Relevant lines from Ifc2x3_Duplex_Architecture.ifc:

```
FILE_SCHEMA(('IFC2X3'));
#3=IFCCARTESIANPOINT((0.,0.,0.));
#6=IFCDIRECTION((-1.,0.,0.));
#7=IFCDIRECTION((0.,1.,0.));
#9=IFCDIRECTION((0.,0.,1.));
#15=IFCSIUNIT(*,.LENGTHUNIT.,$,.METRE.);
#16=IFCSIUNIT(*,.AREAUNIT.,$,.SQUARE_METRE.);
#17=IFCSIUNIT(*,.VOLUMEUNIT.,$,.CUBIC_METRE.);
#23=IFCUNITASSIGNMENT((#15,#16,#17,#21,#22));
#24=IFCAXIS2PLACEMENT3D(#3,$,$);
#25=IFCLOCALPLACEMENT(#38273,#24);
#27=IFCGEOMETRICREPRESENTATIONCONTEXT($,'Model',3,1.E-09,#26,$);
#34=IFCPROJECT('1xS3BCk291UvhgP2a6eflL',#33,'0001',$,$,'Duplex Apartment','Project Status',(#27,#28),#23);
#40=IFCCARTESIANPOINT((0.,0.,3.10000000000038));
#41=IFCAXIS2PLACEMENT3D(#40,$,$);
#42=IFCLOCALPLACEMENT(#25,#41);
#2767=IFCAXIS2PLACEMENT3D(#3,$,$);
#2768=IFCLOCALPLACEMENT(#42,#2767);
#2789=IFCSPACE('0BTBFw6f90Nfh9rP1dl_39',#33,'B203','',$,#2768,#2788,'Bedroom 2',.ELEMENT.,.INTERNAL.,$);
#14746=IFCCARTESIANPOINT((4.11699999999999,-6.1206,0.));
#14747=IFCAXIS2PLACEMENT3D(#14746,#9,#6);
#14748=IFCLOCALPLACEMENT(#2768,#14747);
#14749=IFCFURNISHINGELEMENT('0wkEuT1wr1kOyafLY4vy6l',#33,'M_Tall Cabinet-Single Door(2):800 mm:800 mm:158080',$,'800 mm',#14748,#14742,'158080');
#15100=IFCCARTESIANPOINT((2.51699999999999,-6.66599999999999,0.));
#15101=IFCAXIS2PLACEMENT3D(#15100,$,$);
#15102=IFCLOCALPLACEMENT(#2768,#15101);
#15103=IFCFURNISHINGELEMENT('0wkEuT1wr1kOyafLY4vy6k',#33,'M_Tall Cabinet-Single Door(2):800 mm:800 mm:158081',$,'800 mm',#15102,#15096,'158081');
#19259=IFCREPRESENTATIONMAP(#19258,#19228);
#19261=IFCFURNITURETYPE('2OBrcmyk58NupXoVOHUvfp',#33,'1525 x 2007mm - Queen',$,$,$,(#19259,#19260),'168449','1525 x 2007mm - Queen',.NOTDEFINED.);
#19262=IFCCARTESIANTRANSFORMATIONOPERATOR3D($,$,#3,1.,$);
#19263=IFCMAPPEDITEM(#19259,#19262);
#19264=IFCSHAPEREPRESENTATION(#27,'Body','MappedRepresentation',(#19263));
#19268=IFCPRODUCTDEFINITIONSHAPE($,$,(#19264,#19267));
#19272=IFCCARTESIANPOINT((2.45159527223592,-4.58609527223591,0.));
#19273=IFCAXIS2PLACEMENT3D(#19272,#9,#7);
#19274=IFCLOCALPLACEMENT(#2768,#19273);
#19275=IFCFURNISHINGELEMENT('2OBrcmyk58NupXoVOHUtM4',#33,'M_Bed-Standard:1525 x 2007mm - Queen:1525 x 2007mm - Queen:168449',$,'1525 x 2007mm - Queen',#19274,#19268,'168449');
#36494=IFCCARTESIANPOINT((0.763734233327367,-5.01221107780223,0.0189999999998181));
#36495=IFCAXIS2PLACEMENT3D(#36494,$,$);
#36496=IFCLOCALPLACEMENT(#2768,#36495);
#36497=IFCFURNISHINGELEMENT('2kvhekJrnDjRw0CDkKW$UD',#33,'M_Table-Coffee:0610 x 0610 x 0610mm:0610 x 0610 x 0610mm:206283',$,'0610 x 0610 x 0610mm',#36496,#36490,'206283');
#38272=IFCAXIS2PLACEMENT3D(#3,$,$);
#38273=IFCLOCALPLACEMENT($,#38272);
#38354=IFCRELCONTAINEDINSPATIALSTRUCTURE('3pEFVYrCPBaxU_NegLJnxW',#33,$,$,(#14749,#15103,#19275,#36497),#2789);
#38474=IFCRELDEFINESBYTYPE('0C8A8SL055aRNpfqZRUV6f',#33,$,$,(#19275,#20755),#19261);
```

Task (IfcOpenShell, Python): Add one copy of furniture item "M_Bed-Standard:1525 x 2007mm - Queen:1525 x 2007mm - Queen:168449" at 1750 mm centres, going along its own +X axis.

```python
import ifcopenshell
import ifcopenshell.api.geometry
import ifcopenshell.api.root
import ifcopenshell.util.element
import ifcopenshell.util.placement
import ifcopenshell.util.unit

model = ifcopenshell.open("Ifc2x3_Duplex_Architecture.ifc")
unit_scale = ifcopenshell.util.unit.calculate_unit_scale(model)


def reuse_history(source, copy):
    """copy_class also copies each property set's owner history, people and application; keep the originals."""
    for rel in copy.IsDefinedBy:
        if rel.is_a("IfcRelDefinesByProperties") and (history := rel.RelatingPropertyDefinition.OwnerHistory):
            rel.RelatingPropertyDefinition.OwnerHistory = source.OwnerHistory
            ifcopenshell.util.element.remove_deep2(model, history)


source = model.by_guid("2OBrcmyk58NupXoVOHUtM4")
base = ifcopenshell.util.placement.get_local_placement(source.ObjectPlacement)
step = base[:3, 0] * 1.75 / unit_scale

for i in range(1, 2):
    copy = ifcopenshell.api.root.copy_class(model, product=source)
    copy.Representation = ifcopenshell.util.element.copy_deep(
        model, source.Representation, exclude=["IfcGeometricRepresentationContext", "IfcRepresentationMap"]
    )
    copy.Name = "M_Bed-Standard:1525 x 2007mm - Queen:1525 x 2007mm - Queen"
    copy.Tag = None
    reuse_history(source, copy)
    matrix = base.copy()
    matrix[:3, 3] += i * step
    print("added at", matrix[:3, 3].round(3) + 0.0)
    ifcopenshell.api.geometry.edit_object_placement(model, product=copy, matrix=matrix, is_si=False)

model.write("Ifc2x3_Duplex_Architecture_rev.ifc")
```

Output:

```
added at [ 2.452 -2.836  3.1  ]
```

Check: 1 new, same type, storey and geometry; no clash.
